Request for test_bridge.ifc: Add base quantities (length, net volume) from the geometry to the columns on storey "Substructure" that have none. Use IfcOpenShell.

First a look at what the model holds.

```python
import ifcopenshell
import ifcopenshell.util.element
import ifcopenshell.util.unit

model = ifcopenshell.open("test_bridge.ifc")
print(model.schema)
for unit_type in ("LENGTHUNIT", "AREAUNIT", "VOLUMEUNIT"):
    print(unit_type, ifcopenshell.util.unit.calculate_unit_scale(model, unit_type))
storey = next(s for s in model.by_type("IfcBuildingStorey") if s.Name == "Substructure")
columns = [e for e in ifcopenshell.util.element.get_decomposition(storey) if e.is_a("IfcColumn")]
for e in sorted(columns, key=lambda e: e.id()):
    print(e.id(), e.is_a(), e.Name, list(ifcopenshell.util.element.get_psets(e, qtos_only=True)), sep=" | ")
```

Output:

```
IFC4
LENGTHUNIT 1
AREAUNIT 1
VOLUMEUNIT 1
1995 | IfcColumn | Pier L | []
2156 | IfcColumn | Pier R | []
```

```python
import ifcopenshell
import ifcopenshell.api.pset
import ifcopenshell.geom
import ifcopenshell.util.element
import ifcopenshell.util.shape
import ifcopenshell.util.unit

model = ifcopenshell.open("test_bridge.ifc")
unit_scale = ifcopenshell.util.unit.calculate_unit_scale(model)
volume_scale = ifcopenshell.util.unit.calculate_unit_scale(model, "VOLUMEUNIT")
settings = ifcopenshell.geom.settings()

storey = next(s for s in model.by_type("IfcBuildingStorey") if s.Name == "Substructure")
columns = [e for e in ifcopenshell.util.element.get_decomposition(storey) if e.is_a("IfcColumn")]

for e in sorted(columns, key=lambda e: e.id()):
    if ifcopenshell.util.element.get_psets(e, qtos_only=True, should_inherit=False):
        continue
    # Geometry comes back in metres, in the element's own axes.
    shape = ifcopenshell.geom.create_shape(settings, e)
    values = {
        "Length": ifcopenshell.util.shape.get_z(shape.geometry) / unit_scale,
        "NetVolume": ifcopenshell.util.shape.get_volume(shape.geometry) / volume_scale,
    }
    qto = ifcopenshell.api.pset.add_qto(model, product=e, name="Qto_ColumnBaseQuantities")
    ifcopenshell.api.pset.edit_qto(model, qto=qto, properties=values)
    print(e.id(), {k: round(v, 3) for k, v in values.items()})

model.write("test_bridge-out.ifc")
```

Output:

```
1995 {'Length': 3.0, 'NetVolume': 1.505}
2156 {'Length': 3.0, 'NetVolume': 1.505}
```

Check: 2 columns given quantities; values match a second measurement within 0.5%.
